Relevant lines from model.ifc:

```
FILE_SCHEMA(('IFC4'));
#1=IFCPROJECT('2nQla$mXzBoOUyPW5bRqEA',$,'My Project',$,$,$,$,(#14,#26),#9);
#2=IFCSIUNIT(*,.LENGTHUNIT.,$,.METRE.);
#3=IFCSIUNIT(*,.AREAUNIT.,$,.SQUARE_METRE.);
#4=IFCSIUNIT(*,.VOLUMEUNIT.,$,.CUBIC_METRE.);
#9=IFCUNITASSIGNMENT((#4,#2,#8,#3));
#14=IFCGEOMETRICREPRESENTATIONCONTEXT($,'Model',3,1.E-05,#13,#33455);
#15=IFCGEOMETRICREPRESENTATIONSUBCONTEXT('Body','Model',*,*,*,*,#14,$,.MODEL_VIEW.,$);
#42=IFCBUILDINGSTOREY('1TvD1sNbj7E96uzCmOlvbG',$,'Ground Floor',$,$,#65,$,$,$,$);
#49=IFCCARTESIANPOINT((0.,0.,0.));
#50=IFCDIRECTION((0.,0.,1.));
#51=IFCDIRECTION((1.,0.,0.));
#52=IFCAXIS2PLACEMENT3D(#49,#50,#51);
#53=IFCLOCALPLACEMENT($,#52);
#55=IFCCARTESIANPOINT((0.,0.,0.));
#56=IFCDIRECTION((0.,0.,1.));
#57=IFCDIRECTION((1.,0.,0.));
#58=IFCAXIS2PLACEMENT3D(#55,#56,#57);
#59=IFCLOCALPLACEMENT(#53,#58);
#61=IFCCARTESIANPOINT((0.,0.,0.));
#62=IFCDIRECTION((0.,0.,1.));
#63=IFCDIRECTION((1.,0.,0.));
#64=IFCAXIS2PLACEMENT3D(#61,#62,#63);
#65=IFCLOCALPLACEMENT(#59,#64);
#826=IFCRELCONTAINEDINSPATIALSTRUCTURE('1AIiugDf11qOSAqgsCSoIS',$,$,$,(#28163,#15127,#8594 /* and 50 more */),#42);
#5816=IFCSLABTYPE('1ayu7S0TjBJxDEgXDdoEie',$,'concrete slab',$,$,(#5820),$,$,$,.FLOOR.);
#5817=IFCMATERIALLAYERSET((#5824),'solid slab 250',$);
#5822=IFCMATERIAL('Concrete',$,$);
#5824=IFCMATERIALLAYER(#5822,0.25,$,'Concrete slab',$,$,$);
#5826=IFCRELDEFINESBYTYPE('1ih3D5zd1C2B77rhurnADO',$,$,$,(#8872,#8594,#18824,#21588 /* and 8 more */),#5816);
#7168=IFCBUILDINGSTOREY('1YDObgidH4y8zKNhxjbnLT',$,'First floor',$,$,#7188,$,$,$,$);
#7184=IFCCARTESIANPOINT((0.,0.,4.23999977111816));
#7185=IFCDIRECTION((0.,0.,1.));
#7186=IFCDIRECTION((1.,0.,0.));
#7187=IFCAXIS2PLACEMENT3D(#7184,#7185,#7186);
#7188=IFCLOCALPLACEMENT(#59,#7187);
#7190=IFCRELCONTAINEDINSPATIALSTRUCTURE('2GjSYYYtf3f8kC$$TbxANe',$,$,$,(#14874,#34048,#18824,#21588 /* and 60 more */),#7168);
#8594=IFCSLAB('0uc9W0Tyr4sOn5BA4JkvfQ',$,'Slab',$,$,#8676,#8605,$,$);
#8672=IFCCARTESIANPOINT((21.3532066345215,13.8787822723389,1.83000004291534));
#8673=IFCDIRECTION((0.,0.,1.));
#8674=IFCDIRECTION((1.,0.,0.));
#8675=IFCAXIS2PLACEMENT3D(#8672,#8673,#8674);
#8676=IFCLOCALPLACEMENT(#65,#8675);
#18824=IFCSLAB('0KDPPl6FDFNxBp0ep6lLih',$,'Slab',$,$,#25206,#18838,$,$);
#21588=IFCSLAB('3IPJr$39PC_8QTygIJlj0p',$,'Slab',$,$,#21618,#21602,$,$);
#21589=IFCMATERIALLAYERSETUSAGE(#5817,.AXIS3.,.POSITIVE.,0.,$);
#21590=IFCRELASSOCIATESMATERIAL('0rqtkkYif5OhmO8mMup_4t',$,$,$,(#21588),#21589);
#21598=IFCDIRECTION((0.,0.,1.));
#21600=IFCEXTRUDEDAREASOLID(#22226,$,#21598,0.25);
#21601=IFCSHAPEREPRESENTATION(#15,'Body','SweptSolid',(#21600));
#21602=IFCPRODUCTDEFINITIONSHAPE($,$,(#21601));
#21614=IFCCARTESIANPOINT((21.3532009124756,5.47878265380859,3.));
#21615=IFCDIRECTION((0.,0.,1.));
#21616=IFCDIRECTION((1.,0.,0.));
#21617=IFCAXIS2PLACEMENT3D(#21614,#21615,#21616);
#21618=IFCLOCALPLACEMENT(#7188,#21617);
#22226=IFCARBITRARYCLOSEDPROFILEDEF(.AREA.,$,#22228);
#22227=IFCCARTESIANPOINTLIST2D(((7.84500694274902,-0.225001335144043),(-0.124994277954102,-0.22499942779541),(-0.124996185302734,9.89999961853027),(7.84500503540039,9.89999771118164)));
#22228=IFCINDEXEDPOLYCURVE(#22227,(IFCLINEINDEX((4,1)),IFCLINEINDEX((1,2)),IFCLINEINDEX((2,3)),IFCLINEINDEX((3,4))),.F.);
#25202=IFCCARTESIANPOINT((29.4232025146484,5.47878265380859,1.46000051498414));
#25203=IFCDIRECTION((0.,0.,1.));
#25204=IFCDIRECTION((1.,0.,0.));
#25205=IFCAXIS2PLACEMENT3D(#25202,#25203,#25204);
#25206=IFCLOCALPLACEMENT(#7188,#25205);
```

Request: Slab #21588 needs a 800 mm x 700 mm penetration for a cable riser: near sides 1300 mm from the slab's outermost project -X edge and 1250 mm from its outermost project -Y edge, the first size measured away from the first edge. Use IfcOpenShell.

```python
import numpy as np
import ifcopenshell
import ifcopenshell.api.feature
import ifcopenshell.api.geometry
import ifcopenshell.api.root
import ifcopenshell.geom
import ifcopenshell.util.placement
import ifcopenshell.util.representation
import ifcopenshell.util.shape
import ifcopenshell.util.unit

model = ifcopenshell.open("model.ifc")
unit_scale = ifcopenshell.util.unit.calculate_unit_scale(model)
settings = ifcopenshell.geom.settings()


def volume(element):
    """Net volume in cubic metres, openings subtracted."""
    shape = ifcopenshell.geom.create_shape(settings, element)
    return ifcopenshell.util.shape.get_volume(shape.geometry)


slab = model.by_guid("3IPJr$39PC_8QTygIJlj0p")
before = volume(slab)

# Extent in the slab's own axes, in metres. The edges named are its -X and -Y sides.
slab_shape = ifcopenshell.geom.create_shape(settings, slab)
vertices = ifcopenshell.util.shape.get_vertices(slab_shape.geometry)
x_min, y_min, bottom = vertices.min(axis=0)
top = vertices[:, 2].max()

opening = ifcopenshell.api.root.create_entity(model, ifc_class="IfcOpeningElement", name="Cable riser opening", predefined_type="OPENING")
context = ifcopenshell.util.representation.get_context(model, "Model", "Body", "MODEL_VIEW")
width, depth = 0.8, 0.7
outline = [(0.0, 0.0), (width, 0.0), (width, depth), (0.0, depth), (0.0, 0.0)]
# Overshoot both faces by 50 mm so the cut is clean.
shape = ifcopenshell.api.geometry.add_slab_representation(
    model, context=context, depth=top - bottom + 0.1, polyline=outline
)
ifcopenshell.api.geometry.assign_representation(model, product=opening, representation=shape)

matrix = ifcopenshell.util.placement.get_local_placement(slab.ObjectPlacement)
matrix[:, 3] = matrix @ np.append(np.array([x_min + 1.3, y_min + 1.25, bottom - 0.05]) / unit_scale, 1.0)
ifcopenshell.api.geometry.edit_object_placement(model, product=opening, matrix=matrix, is_si=False)
ifcopenshell.api.feature.add_feature(model, feature=opening, element=slab)

after = volume(slab)

print(f"slab volume {before:.3f} -> {after:.3f} m3")

model.write("model_updated.ifc")
```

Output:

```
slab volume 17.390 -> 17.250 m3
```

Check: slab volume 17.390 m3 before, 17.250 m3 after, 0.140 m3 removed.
